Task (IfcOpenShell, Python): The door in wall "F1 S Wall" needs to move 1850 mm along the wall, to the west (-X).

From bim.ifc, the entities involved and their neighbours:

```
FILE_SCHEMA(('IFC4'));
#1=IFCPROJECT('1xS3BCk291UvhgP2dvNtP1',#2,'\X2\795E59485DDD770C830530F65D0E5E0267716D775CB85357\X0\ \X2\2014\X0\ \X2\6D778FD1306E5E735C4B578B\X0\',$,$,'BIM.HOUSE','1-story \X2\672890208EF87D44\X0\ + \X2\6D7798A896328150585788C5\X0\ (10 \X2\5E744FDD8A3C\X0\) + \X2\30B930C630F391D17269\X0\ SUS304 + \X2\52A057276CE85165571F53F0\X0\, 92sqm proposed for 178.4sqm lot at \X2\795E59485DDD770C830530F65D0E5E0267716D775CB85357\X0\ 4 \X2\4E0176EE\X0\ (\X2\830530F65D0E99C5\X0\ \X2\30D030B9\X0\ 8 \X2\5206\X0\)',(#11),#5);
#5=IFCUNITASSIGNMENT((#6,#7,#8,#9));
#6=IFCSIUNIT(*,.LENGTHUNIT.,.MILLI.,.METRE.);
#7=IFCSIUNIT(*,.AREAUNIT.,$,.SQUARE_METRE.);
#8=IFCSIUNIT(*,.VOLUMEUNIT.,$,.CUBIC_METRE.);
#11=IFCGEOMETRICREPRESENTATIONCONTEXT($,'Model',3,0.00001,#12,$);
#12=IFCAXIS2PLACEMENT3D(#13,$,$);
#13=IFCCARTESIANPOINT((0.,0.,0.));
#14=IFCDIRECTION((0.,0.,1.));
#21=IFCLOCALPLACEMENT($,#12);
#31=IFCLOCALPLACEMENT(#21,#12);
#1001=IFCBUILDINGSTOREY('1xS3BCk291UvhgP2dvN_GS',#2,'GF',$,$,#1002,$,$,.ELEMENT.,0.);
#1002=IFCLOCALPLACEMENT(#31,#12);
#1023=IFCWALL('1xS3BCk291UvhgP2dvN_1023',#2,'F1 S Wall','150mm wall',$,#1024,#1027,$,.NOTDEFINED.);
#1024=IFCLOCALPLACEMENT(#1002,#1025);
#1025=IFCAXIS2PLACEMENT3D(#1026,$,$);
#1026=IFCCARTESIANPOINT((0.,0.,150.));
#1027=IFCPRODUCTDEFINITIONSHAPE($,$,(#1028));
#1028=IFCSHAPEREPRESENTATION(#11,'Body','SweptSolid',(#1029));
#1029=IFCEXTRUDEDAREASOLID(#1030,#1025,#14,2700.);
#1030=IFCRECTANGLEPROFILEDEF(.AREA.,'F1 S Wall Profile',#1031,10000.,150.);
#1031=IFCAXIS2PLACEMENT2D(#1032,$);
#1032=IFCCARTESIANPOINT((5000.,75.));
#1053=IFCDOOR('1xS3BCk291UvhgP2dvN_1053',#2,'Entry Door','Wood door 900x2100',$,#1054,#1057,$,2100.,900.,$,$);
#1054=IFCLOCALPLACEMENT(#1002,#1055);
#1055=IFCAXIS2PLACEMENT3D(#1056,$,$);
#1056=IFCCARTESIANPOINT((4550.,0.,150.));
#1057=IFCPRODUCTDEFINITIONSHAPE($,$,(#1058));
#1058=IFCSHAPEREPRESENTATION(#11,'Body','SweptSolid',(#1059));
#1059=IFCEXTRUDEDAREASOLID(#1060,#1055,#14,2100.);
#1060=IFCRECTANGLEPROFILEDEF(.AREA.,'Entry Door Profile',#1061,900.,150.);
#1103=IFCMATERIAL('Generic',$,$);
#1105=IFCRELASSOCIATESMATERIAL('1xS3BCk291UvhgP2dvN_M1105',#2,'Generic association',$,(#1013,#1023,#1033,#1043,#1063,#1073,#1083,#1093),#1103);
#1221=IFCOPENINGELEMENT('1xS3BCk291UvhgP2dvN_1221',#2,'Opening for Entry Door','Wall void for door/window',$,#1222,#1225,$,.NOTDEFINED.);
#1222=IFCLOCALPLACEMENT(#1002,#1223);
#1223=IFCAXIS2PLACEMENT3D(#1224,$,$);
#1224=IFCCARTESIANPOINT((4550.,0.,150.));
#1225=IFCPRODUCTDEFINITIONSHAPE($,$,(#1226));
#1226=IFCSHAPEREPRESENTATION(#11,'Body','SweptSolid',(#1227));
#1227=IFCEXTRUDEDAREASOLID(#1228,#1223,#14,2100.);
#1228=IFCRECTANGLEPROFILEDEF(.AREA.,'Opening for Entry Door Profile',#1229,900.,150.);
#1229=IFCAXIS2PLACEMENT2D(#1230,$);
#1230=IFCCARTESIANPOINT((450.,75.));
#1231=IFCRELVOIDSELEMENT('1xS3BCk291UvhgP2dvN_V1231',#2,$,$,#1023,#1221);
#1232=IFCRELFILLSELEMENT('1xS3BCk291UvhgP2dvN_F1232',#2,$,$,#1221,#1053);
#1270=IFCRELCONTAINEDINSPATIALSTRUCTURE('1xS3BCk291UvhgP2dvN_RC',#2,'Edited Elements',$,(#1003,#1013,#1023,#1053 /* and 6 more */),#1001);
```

```python
import ifcopenshell
import ifcopenshell.api.geometry
import ifcopenshell.util.placement

model = ifcopenshell.open("bim.ifc")

door = model.by_guid("1xS3BCk291UvhgP2dvN_1053")
opening = door.FillsVoids[0].RelatingOpeningElement
wall = opening.VoidsElements[0].RelatingBuildingElement

wall_matrix = ifcopenshell.util.placement.get_local_placement(wall.ObjectPlacement)
shift = wall_matrix[:3, 0] * -1850.0
before = ifcopenshell.util.placement.get_local_placement(door.ObjectPlacement)[:3, 3].copy()

# The door is not placed relative to its opening, so move both.
for product in (opening, door):
    matrix = ifcopenshell.util.placement.get_local_placement(product.ObjectPlacement)
    matrix[:3, 3] += shift
    ifcopenshell.api.geometry.edit_object_placement(model, product=product, matrix=matrix, is_si=False)

after = ifcopenshell.util.placement.get_local_placement(door.ObjectPlacement)[:3, 3]
print("door moved by", (after - before).round(3) + 0.0)

model.write("bim_updated.ifc")
```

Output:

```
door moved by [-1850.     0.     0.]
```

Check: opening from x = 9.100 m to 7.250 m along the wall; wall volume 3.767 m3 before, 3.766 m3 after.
